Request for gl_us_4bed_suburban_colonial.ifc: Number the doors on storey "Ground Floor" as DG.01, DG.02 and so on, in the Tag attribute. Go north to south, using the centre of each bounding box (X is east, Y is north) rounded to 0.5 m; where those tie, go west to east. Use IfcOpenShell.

First a look at what the model holds.

```python
import ifcopenshell
import ifcopenshell.util.element
import ifcopenshell.util.placement

model = ifcopenshell.open("gl_us_4bed_suburban_colonial.ifc")
print(model.schema)
storey = next(s for s in model.by_type("IfcBuildingStorey") if s.Name == "Ground Floor")
doors = [e for e in ifcopenshell.util.element.get_decomposition(storey) if e.is_a("IfcDoor")]
for e in sorted(doors, key=lambda e: e.id()):
    origin = ifcopenshell.util.placement.get_local_placement(e.ObjectPlacement)[:3, 3]
    print(e.id(), e.Tag, e.Name, origin.round(2) + 0.0, sep=" | ")
```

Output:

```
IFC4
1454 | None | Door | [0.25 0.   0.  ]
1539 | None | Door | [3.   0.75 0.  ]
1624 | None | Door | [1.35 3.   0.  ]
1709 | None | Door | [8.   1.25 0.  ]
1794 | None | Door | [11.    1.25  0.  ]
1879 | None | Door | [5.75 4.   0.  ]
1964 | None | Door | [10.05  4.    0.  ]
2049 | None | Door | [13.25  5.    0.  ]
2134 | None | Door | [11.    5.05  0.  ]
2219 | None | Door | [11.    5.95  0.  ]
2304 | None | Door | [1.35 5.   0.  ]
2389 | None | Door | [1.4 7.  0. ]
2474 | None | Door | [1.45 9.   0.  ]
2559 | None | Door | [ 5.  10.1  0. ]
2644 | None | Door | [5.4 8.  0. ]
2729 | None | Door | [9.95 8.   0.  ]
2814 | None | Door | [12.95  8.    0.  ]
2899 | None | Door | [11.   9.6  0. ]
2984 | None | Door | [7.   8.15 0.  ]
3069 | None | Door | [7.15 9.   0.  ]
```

```python
import ifcopenshell
import ifcopenshell.geom
import ifcopenshell.util.element
import ifcopenshell.util.shape

model = ifcopenshell.open("gl_us_4bed_suburban_colonial.ifc")
settings = ifcopenshell.geom.settings()
settings.set("use-world-coords", True)


def centre(element):
    shape = ifcopenshell.geom.create_shape(settings, element)
    return ifcopenshell.util.shape.get_bbox_centroid(shape.geometry)


storey = next(s for s in model.by_type("IfcBuildingStorey") if s.Name == "Ground Floor")
doors = [e for e in ifcopenshell.util.element.get_decomposition(storey) if e.is_a("IfcDoor")]

# Insertion points can sit at a corner or the storey origin, so sort by the geometry (in metres).
centres = {e: centre(e) for e in doors}
doors.sort(key=lambda e: (-round(centres[e][1] / 0.5), centres[e][0]))

for i, e in enumerate(doors, start=1):
    number = f"DG.{i:02d}"
    e.Tag = number
    print(e.id(), number)

model.write("gl_us_4bed_suburban_colonial_updated.ifc")
```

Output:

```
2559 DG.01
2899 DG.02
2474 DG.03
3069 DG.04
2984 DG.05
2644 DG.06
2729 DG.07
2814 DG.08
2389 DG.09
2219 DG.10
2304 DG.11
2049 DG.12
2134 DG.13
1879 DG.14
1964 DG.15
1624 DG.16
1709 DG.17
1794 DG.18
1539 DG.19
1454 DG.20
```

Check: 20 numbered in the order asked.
